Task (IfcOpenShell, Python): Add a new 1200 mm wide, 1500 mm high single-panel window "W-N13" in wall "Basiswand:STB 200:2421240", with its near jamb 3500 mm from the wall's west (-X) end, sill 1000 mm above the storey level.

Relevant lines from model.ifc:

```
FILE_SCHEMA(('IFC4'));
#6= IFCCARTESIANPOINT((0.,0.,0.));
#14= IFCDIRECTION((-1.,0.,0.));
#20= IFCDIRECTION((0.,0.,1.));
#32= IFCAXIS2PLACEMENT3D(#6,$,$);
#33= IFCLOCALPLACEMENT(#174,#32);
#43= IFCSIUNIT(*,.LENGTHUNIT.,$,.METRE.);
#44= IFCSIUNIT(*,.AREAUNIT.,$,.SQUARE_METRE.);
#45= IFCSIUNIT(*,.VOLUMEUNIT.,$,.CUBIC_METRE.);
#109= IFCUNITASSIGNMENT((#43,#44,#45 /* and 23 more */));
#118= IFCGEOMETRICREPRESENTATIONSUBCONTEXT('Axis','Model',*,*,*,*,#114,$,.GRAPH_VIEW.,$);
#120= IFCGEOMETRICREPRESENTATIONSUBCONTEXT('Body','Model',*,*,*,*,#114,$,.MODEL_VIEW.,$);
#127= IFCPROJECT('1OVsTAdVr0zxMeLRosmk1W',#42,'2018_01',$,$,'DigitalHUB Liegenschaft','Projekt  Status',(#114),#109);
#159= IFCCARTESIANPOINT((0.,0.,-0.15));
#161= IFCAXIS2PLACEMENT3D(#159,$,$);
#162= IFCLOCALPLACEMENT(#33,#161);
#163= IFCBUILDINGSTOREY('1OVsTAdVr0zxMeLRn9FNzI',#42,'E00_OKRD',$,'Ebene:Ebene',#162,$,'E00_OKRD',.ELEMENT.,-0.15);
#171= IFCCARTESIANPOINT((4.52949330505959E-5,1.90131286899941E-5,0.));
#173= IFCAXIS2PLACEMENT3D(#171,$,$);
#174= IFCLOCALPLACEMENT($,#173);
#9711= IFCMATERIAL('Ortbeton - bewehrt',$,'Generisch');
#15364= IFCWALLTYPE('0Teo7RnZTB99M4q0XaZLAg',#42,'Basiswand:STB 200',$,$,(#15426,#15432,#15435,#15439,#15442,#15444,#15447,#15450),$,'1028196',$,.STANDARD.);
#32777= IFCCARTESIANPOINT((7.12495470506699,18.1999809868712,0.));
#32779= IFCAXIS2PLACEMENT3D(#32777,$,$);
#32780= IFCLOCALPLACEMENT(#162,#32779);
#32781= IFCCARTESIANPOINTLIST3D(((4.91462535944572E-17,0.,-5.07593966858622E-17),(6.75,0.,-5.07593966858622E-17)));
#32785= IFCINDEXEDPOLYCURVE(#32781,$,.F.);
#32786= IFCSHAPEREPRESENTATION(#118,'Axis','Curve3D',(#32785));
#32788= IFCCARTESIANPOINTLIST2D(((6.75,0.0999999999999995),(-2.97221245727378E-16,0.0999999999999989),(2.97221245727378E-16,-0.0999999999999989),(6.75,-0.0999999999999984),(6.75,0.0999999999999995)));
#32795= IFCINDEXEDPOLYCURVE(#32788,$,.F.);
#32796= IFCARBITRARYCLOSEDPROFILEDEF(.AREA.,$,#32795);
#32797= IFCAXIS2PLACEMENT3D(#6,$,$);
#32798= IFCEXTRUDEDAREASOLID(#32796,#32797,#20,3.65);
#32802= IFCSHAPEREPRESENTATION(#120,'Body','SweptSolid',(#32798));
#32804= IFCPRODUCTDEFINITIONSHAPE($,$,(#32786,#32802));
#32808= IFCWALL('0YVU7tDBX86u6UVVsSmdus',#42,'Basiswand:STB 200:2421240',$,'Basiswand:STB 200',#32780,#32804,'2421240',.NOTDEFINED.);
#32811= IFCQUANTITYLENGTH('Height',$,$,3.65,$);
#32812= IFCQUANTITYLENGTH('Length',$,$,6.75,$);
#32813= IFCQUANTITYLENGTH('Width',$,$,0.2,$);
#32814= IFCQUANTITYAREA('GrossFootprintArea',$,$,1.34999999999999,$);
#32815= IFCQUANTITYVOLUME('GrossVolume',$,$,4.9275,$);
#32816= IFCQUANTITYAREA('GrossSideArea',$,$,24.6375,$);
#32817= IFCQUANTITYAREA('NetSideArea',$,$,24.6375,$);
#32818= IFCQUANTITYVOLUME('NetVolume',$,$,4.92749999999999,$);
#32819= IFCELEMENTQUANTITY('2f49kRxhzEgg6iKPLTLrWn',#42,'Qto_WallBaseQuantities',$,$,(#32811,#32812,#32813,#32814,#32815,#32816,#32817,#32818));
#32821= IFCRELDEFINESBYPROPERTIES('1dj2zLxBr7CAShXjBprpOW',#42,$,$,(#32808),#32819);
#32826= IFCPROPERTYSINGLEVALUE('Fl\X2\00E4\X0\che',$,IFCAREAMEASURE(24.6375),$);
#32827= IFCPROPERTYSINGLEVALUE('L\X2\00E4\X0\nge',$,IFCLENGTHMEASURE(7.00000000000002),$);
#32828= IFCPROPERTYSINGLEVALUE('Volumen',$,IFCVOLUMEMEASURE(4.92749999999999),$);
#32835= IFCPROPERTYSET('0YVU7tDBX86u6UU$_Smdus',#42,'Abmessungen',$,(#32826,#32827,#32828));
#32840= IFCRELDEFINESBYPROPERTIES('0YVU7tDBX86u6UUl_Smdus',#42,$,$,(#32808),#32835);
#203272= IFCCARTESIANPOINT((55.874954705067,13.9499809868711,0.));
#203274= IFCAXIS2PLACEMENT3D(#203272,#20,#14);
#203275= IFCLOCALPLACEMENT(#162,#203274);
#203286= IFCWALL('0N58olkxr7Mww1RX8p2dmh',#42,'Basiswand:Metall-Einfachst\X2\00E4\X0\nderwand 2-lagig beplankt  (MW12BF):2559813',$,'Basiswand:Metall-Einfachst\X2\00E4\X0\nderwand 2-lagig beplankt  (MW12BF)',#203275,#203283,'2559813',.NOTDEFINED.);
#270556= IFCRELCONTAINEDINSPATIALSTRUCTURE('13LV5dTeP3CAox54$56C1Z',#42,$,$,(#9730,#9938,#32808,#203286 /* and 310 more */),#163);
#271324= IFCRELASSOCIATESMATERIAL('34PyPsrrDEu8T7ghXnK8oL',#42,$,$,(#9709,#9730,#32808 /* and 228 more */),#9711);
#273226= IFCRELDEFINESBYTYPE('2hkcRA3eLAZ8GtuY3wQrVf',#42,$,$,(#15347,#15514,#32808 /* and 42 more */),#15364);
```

```python
import numpy as np
import ifcopenshell
import ifcopenshell.api.feature
import ifcopenshell.api.geometry
import ifcopenshell.api.pset
import ifcopenshell.api.root
import ifcopenshell.api.spatial
import ifcopenshell.geom
import ifcopenshell.util.element
import ifcopenshell.util.placement
import ifcopenshell.util.representation
import ifcopenshell.util.shape
import ifcopenshell.util.unit

model = ifcopenshell.open("model.ifc")
unit_scale = ifcopenshell.util.unit.calculate_unit_scale(model)
area_scale = ifcopenshell.util.unit.calculate_unit_scale(model, "AREAUNIT")
volume_scale = ifcopenshell.util.unit.calculate_unit_scale(model, "VOLUMEUNIT")
settings = ifcopenshell.geom.settings()


def volume(element):
    """Net volume in cubic metres, openings subtracted."""
    shape = ifcopenshell.geom.create_shape(settings, element)
    return ifcopenshell.util.shape.get_volume(shape.geometry)


wall = model.by_id(32808)
storey = ifcopenshell.util.element.get_container(wall, ifc_class="IfcBuildingStorey")
context = ifcopenshell.util.representation.get_context(model, "Model", "Body", "MODEL_VIEW")
before = volume(wall)

width, height, from_end, sill = 1.2, 1.5, 3.5, 1  # metres

# The wall runs along its own X axis, and the end named is its -X end.
wall_shape = ifcopenshell.geom.create_shape(settings, wall)
x, y, z = ifcopenshell.util.shape.get_vertices(wall_shape.geometry).T
start = x.min() + from_end
face, thickness = float(y.min()), float(y.max() - y.min())
wall_matrix = ifcopenshell.util.placement.get_local_placement(wall.ObjectPlacement)
level = ifcopenshell.util.placement.get_local_placement(storey.ObjectPlacement)[2, 3]


def in_wall(x, y):
    """Placement at x, y metres in the wall's axes, at sill height."""
    matrix = wall_matrix.copy()
    matrix[:, 3] = wall_matrix @ np.array([x / unit_scale, y / unit_scale, 0.0, 1.0])
    matrix[2, 3] = level + sill / unit_scale
    return matrix


# Opening: a box that overshoots both wall faces by 50 mm.
opening = ifcopenshell.api.root.create_entity(model, ifc_class="IfcOpeningElement", predefined_type="OPENING")
box = ifcopenshell.api.geometry.add_wall_representation(
    model, context=context, length=width, height=height, thickness=thickness + 0.1
)
ifcopenshell.api.geometry.assign_representation(model, product=opening, representation=box)
ifcopenshell.api.geometry.edit_object_placement(model, product=opening, matrix=in_wall(start, face - 0.05), is_si=False)
ifcopenshell.api.feature.add_feature(model, feature=opening, element=wall)

window = ifcopenshell.api.root.create_entity(model, ifc_class="IfcWindow", name="W-N13", predefined_type="WINDOW")
window.OverallWidth, window.OverallHeight = width / unit_scale, height / unit_scale
window.PartitioningType = "SINGLE_PANEL"
body = ifcopenshell.api.geometry.add_window_representation(
    model,
    context=context,
    overall_width=window.OverallWidth,
    overall_height=window.OverallHeight,
    partition_type="SINGLE_PANEL",
)
ifcopenshell.api.geometry.assign_representation(model, product=window, representation=body)
ifcopenshell.api.spatial.assign_container(model, products=[window], relating_structure=storey)
ifcopenshell.api.feature.add_filling(model, opening=opening, element=window)

# Centre the window in the wall's thickness.
ifcopenshell.api.geometry.edit_object_placement(model, product=window, matrix=in_wall(start, face), is_si=False)
window_shape = ifcopenshell.geom.create_shape(settings, window)
depth = ifcopenshell.util.shape.get_vertices(window_shape.geometry)[:, 1]
offset = face + thickness / 2 - (depth.min() + depth.max()) / 2
ifcopenshell.api.geometry.edit_object_placement(model, product=window, matrix=in_wall(start, offset), is_si=False)

after = volume(wall)

# Update the wall's stored quantities.
qto = model.by_id(ifcopenshell.util.element.get_pset(wall, "Qto_WallBaseQuantities", should_inherit=False)["id"])
ifcopenshell.api.pset.edit_qto(model, qto=qto, properties={
    "NetSideArea": after / thickness / area_scale,
    "NetVolume": after / volume_scale,
})
pset = model.by_id(ifcopenshell.util.element.get_pset(wall, "Abmessungen", should_inherit=False)["id"])
ifcopenshell.api.pset.edit_pset(model, pset=pset, properties={
    "Fläche": model.create_entity("IfcAreaMeasure", after / thickness / area_scale),
    "Volumen": model.create_entity("IfcVolumeMeasure", after / volume_scale),
})

print(f"wall volume {before:.3f} -> {after:.3f} m3")

model.write("model_v2.ifc")
```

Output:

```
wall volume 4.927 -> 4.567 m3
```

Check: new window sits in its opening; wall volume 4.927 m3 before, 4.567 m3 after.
